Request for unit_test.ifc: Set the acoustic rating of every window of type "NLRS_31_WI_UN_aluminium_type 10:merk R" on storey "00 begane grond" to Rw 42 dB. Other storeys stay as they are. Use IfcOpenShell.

First a look at what the model holds.

```python
import ifcopenshell
import ifcopenshell.util.element

model = ifcopenshell.open("unit_test.ifc")
print(model.schema)
storey = next(s for s in model.by_type("IfcBuildingStorey") if s.Name == "00 begane grond")
windows = [e for e in ifcopenshell.util.element.get_decomposition(storey) if e.is_a("IfcWindow")]
seen = {}
for e in windows:
    element_type = ifcopenshell.util.element.get_type(e)
    key = (element_type.Name if element_type != e and element_type else None, ifcopenshell.util.element.get_pset(e, "Pset_WindowCommon", "AcousticRating"))
    seen[key] = seen.get(key, 0) + 1
for (name, value), count in sorted(seen.items(), key=str):
    print(count, "x", name, "|", value)
```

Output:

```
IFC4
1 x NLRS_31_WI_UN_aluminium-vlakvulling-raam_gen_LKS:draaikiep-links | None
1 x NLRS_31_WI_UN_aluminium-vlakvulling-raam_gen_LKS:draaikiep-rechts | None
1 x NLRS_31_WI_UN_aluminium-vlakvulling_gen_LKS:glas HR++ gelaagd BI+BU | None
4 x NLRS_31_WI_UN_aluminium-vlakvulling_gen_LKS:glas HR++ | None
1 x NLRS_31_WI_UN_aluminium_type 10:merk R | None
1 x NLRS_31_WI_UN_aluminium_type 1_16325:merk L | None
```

```python
import ifcopenshell
import ifcopenshell.api.pset
import ifcopenshell.util.element

model = ifcopenshell.open("unit_test.ifc")

storey = next(s for s in model.by_type("IfcBuildingStorey") if s.Name == "00 begane grond")
windows = [e for e in ifcopenshell.util.element.get_decomposition(storey) if e.is_a("IfcWindow")]

count = 0
for e in windows:
    element_type = ifcopenshell.util.element.get_type(e)
    if element_type in (None, e) or element_type.Name != "NLRS_31_WI_UN_aluminium_type 10:merk R":
        continue
    # add_pset returns the element's existing set when there is one.
    pset = ifcopenshell.api.pset.add_pset(model, product=e, name="Pset_WindowCommon")
    ifcopenshell.api.pset.edit_pset(model, pset=pset, properties={"AcousticRating": "Rw 42 dB"})
    count += 1

print(count, "windows updated")

model.write("unit_test_rev.ifc")
```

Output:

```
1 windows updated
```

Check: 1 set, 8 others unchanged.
